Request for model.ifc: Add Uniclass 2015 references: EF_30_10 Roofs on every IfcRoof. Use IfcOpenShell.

First a look at what the model holds.

```python
import ifcopenshell

model = ifcopenshell.open("model.ifc")
print(model.schema)
print("classifications:", [c.Name for c in model.by_type("IfcClassification")])
for ifc_class in ("IfcDoor", "IfcRoof", "IfcStair", "IfcWall", "IfcWindow"):
    print(ifc_class, len(model.by_type(ifc_class)))
```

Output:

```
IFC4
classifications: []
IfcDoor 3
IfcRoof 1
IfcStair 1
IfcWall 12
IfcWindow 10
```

```python
import ifcopenshell
import ifcopenshell.api.classification

model = ifcopenshell.open("model.ifc")

system = ifcopenshell.api.classification.add_classification(model, classification="Uniclass 2015")

codes = {
    "IfcRoof": ("EF_30_10", "Roofs"),
}
for ifc_class, (code, name) in codes.items():
    products = model.by_type(ifc_class)
    ifcopenshell.api.classification.add_reference(
        model, products=products, classification=system, identification=code, name=name
    )
    print(code, len(products))

model.write("model-out.ifc")
```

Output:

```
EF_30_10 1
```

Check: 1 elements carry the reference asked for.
